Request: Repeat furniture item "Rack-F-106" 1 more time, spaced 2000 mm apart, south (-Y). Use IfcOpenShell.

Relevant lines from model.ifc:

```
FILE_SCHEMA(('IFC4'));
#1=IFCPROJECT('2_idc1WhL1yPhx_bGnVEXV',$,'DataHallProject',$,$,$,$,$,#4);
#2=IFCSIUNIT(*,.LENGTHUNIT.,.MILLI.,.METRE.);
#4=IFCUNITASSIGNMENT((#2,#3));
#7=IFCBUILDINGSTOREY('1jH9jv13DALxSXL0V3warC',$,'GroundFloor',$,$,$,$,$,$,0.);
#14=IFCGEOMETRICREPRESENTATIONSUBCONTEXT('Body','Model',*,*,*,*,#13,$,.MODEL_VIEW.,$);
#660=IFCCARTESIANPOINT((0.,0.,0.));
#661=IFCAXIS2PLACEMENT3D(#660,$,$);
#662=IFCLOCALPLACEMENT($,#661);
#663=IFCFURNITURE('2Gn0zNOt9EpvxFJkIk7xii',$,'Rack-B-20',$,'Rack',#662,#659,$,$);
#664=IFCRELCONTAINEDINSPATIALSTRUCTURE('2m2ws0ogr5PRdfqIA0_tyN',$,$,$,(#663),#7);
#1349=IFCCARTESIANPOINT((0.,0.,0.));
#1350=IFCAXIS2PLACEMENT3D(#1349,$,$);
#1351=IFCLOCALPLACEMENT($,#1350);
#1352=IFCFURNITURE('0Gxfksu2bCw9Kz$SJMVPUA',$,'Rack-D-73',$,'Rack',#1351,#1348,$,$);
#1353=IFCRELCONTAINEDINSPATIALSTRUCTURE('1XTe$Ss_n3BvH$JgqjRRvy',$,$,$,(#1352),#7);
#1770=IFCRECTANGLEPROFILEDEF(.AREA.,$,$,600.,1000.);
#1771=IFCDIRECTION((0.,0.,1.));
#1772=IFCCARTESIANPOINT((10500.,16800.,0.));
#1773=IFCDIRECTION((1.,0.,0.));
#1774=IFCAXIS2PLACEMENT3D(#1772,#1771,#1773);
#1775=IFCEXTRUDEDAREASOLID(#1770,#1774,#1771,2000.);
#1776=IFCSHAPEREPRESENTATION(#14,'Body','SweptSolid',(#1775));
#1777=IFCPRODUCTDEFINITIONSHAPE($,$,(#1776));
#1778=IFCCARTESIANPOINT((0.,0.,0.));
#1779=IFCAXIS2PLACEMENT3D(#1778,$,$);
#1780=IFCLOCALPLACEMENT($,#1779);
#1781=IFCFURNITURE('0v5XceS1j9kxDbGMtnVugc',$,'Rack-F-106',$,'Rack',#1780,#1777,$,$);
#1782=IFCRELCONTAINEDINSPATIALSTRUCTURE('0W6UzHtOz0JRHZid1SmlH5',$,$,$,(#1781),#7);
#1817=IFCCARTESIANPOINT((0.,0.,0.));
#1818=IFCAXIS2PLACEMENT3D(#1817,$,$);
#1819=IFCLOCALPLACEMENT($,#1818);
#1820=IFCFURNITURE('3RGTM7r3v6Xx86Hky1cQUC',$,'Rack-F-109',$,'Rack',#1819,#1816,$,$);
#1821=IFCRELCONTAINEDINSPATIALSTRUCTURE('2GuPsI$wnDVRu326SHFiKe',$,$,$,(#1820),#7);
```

```python
import numpy as np
import ifcopenshell
import ifcopenshell.api.geometry
import ifcopenshell.api.root
import ifcopenshell.util.element
import ifcopenshell.util.placement
import ifcopenshell.util.unit

model = ifcopenshell.open("model.ifc")
unit_scale = ifcopenshell.util.unit.calculate_unit_scale(model)

source = model.by_guid("0v5XceS1j9kxDbGMtnVugc")
base = ifcopenshell.util.placement.get_local_placement(source.ObjectPlacement)
step = np.array([0.0, -1.0, 0.0]) * 2 / unit_scale

for i in range(1, 2):
    copy = ifcopenshell.api.root.copy_class(model, product=source)
    copy.Representation = ifcopenshell.util.element.copy_deep(
        model, source.Representation, exclude=["IfcGeometricRepresentationContext", "IfcRepresentationMap"]
    )
    matrix = base.copy()
    matrix[:3, 3] += i * step
    print("added at", matrix[:3, 3].round(3) + 0.0)
    ifcopenshell.api.geometry.edit_object_placement(model, product=copy, matrix=matrix, is_si=False)

model.write("model_updated.ifc")
```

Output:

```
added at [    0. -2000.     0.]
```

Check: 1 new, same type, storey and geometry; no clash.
